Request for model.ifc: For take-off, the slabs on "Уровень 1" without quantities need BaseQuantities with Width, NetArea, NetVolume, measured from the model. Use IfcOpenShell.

First a look at what the model holds.

```python
import ifcopenshell
import ifcopenshell.util.element
import ifcopenshell.util.unit

model = ifcopenshell.open("model.ifc")
print(model.schema)
for unit_type in ("LENGTHUNIT", "AREAUNIT", "VOLUMEUNIT"):
    print(unit_type, ifcopenshell.util.unit.calculate_unit_scale(model, unit_type))
storey = next(s for s in model.by_type("IfcBuildingStorey") if s.Name == "Уровень 1")
slabs = [e for e in ifcopenshell.util.element.get_decomposition(storey) if e.is_a("IfcSlab")]
for e in sorted(slabs, key=lambda e: e.id()):
    print(e.id(), e.is_a(), e.Name, list(ifcopenshell.util.element.get_psets(e, qtos_only=True)), sep=" | ")
```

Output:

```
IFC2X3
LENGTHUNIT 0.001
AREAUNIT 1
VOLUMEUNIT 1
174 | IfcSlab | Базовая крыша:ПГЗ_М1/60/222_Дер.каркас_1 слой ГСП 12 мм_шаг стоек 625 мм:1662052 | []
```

```python
import ifcopenshell
import ifcopenshell.api.pset
import ifcopenshell.geom
import ifcopenshell.util.element
import ifcopenshell.util.shape
import ifcopenshell.util.unit

model = ifcopenshell.open("model.ifc")
unit_scale = ifcopenshell.util.unit.calculate_unit_scale(model)
area_scale = ifcopenshell.util.unit.calculate_unit_scale(model, "AREAUNIT")
volume_scale = ifcopenshell.util.unit.calculate_unit_scale(model, "VOLUMEUNIT")
settings = ifcopenshell.geom.settings()

storey = next(s for s in model.by_type("IfcBuildingStorey") if s.Name == "Уровень 1")
slabs = [e for e in ifcopenshell.util.element.get_decomposition(storey) if e.is_a("IfcSlab")]

for e in sorted(slabs, key=lambda e: e.id()):
    if ifcopenshell.util.element.get_psets(e, qtos_only=True, should_inherit=False):
        continue
    # Geometry comes back in metres, in the element's own axes.
    shape = ifcopenshell.geom.create_shape(settings, e)
    values = {
        "Width": ifcopenshell.util.shape.get_z(shape.geometry) / unit_scale,
        "NetArea": ifcopenshell.util.shape.get_footprint_area(shape.geometry) / area_scale,
        "NetVolume": ifcopenshell.util.shape.get_volume(shape.geometry) / volume_scale,
    }
    qto = ifcopenshell.api.pset.add_qto(model, product=e, name="BaseQuantities")
    ifcopenshell.api.pset.edit_qto(model, qto=qto, properties=values)
    print(e.id(), {k: round(v, 3) for k, v in values.items()})

model.write("model-out.ifc")
```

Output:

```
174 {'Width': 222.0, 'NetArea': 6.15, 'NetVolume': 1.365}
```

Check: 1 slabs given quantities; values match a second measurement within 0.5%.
